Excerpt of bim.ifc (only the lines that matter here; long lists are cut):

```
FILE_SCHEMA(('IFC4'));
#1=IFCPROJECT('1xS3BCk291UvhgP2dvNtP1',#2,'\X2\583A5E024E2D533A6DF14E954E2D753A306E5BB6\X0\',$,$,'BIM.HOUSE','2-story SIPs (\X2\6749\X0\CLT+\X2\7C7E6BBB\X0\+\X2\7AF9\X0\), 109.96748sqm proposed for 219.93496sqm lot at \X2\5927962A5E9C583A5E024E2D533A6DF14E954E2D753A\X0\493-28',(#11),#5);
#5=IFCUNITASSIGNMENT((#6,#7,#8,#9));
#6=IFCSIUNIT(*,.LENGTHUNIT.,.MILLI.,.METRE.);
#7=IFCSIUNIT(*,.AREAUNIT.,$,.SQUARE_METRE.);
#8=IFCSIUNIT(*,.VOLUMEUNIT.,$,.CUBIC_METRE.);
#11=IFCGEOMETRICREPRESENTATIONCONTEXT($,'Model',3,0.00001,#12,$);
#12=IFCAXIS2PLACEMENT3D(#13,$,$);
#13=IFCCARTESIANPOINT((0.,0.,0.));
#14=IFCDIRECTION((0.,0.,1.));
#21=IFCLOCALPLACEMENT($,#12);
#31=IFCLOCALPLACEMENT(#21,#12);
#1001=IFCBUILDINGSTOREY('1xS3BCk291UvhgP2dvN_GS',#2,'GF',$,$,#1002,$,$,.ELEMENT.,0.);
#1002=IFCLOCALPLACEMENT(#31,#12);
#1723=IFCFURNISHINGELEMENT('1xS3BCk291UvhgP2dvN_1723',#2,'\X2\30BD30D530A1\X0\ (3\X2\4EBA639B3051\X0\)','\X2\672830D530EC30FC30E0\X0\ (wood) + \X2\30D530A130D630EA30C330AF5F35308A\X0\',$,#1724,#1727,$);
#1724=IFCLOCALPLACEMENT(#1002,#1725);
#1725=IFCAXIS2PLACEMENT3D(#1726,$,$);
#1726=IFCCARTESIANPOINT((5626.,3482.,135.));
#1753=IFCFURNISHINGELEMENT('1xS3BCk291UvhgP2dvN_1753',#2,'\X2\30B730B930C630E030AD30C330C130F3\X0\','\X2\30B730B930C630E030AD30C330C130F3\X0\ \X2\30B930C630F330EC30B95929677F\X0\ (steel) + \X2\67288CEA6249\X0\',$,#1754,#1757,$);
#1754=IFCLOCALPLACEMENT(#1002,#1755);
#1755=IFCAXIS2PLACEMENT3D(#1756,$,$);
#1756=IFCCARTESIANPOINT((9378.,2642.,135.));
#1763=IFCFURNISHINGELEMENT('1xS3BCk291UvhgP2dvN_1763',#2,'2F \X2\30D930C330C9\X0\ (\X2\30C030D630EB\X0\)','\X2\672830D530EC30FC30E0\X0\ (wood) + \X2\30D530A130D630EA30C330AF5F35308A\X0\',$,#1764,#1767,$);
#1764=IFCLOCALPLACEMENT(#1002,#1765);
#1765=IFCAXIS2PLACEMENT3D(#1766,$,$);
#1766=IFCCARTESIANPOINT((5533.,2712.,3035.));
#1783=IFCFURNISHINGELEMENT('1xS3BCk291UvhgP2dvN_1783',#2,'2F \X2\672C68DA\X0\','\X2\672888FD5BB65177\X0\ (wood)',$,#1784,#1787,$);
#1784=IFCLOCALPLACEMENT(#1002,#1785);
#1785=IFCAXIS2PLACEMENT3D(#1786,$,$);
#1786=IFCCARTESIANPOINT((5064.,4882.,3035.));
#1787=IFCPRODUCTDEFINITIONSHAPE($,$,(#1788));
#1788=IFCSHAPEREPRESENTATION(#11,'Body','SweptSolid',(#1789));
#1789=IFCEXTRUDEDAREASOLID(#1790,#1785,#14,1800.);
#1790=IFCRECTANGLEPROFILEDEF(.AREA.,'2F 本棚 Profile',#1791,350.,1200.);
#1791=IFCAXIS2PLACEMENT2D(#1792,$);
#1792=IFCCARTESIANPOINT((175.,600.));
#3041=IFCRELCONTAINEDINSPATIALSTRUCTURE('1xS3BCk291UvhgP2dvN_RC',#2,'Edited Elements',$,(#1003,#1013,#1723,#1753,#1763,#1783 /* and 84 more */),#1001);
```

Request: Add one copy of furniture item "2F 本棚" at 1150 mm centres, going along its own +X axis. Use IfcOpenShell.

```python
import ifcopenshell
import ifcopenshell.api.geometry
import ifcopenshell.api.root
import ifcopenshell.util.element
import ifcopenshell.util.placement
import ifcopenshell.util.unit

model = ifcopenshell.open("bim.ifc")
unit_scale = ifcopenshell.util.unit.calculate_unit_scale(model)


def reuse_history(source, copy):
    """copy_class also copies each property set's owner history, people and application; keep the originals."""
    for rel in copy.IsDefinedBy:
        if rel.is_a("IfcRelDefinesByProperties") and (history := rel.RelatingPropertyDefinition.OwnerHistory):
            rel.RelatingPropertyDefinition.OwnerHistory = source.OwnerHistory
            ifcopenshell.util.element.remove_deep2(model, history)


source = model.by_id(1783)
base = ifcopenshell.util.placement.get_local_placement(source.ObjectPlacement)
step = base[:3, 0] * 1.15 / unit_scale

for i in range(1, 2):
    copy = ifcopenshell.api.root.copy_class(model, product=source)
    copy.Representation = ifcopenshell.util.element.copy_deep(
        model, source.Representation, exclude=["IfcGeometricRepresentationContext", "IfcRepresentationMap"]
    )
    reuse_history(source, copy)
    matrix = base.copy()
    matrix[:3, 3] += i * step
    print("added at", matrix[:3, 3].round(3) + 0.0)
    ifcopenshell.api.geometry.edit_object_placement(model, product=copy, matrix=matrix, is_si=False)

model.write("bim_v2.ifc")
```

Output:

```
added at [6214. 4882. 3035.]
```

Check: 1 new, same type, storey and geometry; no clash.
